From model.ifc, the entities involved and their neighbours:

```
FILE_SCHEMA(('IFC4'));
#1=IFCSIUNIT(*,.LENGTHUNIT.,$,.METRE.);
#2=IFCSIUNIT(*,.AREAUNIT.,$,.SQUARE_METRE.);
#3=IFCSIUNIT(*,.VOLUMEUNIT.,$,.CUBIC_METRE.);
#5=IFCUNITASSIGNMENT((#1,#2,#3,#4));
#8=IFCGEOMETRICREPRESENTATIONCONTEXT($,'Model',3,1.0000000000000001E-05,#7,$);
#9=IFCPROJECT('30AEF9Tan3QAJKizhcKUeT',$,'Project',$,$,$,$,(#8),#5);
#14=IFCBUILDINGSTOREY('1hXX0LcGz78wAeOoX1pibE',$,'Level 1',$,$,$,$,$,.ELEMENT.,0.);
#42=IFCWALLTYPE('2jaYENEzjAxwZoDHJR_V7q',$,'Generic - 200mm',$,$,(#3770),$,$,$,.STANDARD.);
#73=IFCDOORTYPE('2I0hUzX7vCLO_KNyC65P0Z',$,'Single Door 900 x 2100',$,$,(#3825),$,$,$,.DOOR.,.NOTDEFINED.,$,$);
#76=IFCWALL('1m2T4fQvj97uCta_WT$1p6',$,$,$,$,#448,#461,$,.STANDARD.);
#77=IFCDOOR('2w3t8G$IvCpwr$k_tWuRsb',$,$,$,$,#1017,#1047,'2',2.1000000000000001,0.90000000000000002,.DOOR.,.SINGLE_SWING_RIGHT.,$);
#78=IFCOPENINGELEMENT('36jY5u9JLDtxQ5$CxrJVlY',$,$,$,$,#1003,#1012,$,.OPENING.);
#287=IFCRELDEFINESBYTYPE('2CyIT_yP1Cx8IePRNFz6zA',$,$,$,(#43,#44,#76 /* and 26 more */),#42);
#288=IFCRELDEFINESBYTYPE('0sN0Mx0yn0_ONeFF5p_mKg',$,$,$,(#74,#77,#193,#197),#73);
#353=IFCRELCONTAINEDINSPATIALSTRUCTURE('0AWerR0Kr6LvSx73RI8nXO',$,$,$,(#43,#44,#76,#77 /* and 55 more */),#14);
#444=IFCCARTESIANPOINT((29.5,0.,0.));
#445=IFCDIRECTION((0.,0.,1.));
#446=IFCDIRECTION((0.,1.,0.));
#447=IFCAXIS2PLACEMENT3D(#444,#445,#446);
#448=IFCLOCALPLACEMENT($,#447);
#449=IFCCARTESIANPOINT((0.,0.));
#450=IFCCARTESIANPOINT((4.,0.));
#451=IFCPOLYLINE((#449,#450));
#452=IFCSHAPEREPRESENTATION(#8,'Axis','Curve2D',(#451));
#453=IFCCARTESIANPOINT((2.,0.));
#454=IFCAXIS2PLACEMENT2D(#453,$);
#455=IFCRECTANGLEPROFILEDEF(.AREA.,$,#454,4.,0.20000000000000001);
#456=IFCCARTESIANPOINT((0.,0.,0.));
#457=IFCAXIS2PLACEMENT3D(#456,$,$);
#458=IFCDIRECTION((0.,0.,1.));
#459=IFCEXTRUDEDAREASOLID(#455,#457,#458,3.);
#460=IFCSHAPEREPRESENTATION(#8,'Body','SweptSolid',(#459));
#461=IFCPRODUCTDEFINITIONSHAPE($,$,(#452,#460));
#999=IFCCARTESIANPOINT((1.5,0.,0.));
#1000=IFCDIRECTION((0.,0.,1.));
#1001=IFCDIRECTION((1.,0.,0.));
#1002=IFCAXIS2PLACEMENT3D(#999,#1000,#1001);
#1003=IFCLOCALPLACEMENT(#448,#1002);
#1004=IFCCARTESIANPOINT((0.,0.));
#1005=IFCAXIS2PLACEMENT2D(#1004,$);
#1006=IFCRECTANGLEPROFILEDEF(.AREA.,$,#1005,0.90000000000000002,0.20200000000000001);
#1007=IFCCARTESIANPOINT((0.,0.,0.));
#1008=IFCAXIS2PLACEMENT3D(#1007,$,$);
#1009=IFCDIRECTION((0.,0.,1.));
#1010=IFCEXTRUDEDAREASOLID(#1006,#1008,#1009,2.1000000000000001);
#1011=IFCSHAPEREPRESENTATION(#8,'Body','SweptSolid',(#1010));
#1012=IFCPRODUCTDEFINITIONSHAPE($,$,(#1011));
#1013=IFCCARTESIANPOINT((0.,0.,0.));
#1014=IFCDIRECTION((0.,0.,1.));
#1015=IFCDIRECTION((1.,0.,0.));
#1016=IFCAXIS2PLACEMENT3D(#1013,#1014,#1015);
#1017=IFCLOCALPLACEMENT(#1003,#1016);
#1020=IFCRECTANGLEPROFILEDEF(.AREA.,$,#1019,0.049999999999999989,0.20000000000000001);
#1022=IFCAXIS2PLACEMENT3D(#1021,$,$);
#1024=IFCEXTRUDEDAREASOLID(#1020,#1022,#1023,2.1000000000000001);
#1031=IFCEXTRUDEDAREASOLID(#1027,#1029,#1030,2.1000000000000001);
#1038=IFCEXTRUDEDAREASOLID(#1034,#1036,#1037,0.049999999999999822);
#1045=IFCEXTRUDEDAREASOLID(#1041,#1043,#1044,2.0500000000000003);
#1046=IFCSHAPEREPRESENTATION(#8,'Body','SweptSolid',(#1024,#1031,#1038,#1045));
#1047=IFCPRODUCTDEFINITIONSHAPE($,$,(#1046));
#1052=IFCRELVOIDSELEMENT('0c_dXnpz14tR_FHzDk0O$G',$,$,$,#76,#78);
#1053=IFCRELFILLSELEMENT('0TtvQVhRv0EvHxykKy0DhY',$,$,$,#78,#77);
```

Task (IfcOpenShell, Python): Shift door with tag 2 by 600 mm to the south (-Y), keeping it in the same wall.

```python
import ifcopenshell
import ifcopenshell.api.geometry
import ifcopenshell.util.placement
import ifcopenshell.util.unit

model = ifcopenshell.open("model.ifc")
unit_scale = ifcopenshell.util.unit.calculate_unit_scale(model)

door = model.by_id(77)
opening = door.FillsVoids[0].RelatingOpeningElement
wall = opening.VoidsElements[0].RelatingBuildingElement

wall_matrix = ifcopenshell.util.placement.get_local_placement(wall.ObjectPlacement)
shift = wall_matrix[:3, 0] * -0.6 / unit_scale
before = ifcopenshell.util.placement.get_local_placement(door.ObjectPlacement)[:3, 3].copy()

# The door is placed relative to its opening, so it follows when the opening moves.
matrix = ifcopenshell.util.placement.get_local_placement(opening.ObjectPlacement)
matrix[:3, 3] += shift
ifcopenshell.api.geometry.edit_object_placement(
    model, product=opening, matrix=matrix, is_si=False, should_transform_children=True
)

after = ifcopenshell.util.placement.get_local_placement(door.ObjectPlacement)[:3, 3]
print("door moved by", (after - before).round(3) + 0.0)

model.write("model_updated.ifc")
```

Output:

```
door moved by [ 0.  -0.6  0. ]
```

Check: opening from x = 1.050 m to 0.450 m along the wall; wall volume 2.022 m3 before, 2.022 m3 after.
